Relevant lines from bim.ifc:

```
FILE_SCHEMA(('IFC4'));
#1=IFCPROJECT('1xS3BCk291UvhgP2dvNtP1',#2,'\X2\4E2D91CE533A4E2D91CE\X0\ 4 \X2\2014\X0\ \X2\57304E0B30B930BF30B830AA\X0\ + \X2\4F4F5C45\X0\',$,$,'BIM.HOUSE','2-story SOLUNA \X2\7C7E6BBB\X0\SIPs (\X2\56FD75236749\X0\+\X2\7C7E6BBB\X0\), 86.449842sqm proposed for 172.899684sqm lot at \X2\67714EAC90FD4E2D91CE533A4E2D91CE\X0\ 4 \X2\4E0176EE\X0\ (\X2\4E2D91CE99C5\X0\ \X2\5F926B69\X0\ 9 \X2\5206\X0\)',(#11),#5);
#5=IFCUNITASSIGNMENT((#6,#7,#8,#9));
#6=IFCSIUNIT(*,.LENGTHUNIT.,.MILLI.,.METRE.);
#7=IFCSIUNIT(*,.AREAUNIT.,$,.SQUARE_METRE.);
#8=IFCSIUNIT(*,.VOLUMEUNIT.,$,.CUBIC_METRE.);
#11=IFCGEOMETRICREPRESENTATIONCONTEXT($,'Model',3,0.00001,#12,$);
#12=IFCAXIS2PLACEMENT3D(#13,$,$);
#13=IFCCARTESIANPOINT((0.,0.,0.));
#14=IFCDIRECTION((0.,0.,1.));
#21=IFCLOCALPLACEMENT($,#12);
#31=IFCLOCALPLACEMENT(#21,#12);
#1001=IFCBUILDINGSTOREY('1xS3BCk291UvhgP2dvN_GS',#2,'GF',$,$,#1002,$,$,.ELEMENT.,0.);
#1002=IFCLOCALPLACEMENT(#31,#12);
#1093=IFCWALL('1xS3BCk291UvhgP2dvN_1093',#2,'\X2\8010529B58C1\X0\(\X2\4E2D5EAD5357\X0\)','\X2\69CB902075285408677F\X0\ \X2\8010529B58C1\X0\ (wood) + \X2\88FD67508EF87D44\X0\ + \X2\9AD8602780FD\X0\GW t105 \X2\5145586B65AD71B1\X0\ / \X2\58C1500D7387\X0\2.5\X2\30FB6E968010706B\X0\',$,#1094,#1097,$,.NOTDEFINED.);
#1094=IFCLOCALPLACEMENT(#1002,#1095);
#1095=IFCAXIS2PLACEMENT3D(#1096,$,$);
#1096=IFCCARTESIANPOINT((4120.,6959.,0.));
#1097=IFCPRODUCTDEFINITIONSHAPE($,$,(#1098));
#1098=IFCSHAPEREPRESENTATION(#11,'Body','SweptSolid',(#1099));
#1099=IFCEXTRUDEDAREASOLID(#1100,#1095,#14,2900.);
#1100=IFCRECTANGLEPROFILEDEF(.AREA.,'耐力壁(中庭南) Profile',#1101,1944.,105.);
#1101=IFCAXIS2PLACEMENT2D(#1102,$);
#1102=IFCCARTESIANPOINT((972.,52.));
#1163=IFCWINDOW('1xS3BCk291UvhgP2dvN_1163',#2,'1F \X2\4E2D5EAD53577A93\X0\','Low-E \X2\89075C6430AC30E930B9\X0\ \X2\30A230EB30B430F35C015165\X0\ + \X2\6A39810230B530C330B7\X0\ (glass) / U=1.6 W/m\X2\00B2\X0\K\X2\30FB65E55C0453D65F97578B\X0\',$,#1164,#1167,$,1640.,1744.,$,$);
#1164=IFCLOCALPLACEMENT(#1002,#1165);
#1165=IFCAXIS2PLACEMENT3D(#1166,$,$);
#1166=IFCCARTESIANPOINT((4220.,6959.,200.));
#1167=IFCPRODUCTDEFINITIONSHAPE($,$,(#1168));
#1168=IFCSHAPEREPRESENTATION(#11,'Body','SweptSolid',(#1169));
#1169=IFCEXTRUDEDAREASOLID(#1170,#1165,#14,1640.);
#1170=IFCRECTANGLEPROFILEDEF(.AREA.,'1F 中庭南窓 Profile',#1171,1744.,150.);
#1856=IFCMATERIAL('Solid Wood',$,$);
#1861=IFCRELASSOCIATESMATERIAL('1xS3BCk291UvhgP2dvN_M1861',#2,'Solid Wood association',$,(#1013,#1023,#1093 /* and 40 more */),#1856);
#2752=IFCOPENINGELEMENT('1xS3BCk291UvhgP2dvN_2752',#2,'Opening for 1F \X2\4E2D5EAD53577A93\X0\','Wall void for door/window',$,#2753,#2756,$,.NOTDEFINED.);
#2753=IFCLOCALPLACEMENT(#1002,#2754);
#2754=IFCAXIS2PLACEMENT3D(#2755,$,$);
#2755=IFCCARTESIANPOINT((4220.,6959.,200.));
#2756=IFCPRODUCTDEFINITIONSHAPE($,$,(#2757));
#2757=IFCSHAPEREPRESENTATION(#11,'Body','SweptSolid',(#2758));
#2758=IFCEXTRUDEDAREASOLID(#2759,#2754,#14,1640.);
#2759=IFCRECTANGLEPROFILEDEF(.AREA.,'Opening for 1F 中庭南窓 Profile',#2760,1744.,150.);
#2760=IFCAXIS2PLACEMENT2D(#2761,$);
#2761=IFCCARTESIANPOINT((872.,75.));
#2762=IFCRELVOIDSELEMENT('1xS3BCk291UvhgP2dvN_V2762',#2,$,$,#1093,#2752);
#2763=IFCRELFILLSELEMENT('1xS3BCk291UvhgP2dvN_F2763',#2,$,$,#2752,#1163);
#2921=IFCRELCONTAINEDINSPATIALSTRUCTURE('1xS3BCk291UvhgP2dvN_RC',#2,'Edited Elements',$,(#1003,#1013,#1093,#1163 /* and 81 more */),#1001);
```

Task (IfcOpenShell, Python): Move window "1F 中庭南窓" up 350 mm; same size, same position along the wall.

```python
import numpy as np
import ifcopenshell
import ifcopenshell.api.geometry
import ifcopenshell.util.placement
import ifcopenshell.util.unit

model = ifcopenshell.open("bim.ifc")
unit_scale = ifcopenshell.util.unit.calculate_unit_scale(model)

window = model.by_id(1163)
opening = window.FillsVoids[0].RelatingOpeningElement
dz = 0.35 / unit_scale

shift = np.array([0.0, 0.0, dz])
# The window is not placed relative to its opening, so move both.
for product in (opening, window):
    matrix = ifcopenshell.util.placement.get_local_placement(product.ObjectPlacement)
    matrix[:3, 3] += shift
    ifcopenshell.api.geometry.edit_object_placement(model, product=product, matrix=matrix, is_si=False)

print(f"moved by {dz * unit_scale:+.3f} m")

model.write("bim_edited.ifc")
```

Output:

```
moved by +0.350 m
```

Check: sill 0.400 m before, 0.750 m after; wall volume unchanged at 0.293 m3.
